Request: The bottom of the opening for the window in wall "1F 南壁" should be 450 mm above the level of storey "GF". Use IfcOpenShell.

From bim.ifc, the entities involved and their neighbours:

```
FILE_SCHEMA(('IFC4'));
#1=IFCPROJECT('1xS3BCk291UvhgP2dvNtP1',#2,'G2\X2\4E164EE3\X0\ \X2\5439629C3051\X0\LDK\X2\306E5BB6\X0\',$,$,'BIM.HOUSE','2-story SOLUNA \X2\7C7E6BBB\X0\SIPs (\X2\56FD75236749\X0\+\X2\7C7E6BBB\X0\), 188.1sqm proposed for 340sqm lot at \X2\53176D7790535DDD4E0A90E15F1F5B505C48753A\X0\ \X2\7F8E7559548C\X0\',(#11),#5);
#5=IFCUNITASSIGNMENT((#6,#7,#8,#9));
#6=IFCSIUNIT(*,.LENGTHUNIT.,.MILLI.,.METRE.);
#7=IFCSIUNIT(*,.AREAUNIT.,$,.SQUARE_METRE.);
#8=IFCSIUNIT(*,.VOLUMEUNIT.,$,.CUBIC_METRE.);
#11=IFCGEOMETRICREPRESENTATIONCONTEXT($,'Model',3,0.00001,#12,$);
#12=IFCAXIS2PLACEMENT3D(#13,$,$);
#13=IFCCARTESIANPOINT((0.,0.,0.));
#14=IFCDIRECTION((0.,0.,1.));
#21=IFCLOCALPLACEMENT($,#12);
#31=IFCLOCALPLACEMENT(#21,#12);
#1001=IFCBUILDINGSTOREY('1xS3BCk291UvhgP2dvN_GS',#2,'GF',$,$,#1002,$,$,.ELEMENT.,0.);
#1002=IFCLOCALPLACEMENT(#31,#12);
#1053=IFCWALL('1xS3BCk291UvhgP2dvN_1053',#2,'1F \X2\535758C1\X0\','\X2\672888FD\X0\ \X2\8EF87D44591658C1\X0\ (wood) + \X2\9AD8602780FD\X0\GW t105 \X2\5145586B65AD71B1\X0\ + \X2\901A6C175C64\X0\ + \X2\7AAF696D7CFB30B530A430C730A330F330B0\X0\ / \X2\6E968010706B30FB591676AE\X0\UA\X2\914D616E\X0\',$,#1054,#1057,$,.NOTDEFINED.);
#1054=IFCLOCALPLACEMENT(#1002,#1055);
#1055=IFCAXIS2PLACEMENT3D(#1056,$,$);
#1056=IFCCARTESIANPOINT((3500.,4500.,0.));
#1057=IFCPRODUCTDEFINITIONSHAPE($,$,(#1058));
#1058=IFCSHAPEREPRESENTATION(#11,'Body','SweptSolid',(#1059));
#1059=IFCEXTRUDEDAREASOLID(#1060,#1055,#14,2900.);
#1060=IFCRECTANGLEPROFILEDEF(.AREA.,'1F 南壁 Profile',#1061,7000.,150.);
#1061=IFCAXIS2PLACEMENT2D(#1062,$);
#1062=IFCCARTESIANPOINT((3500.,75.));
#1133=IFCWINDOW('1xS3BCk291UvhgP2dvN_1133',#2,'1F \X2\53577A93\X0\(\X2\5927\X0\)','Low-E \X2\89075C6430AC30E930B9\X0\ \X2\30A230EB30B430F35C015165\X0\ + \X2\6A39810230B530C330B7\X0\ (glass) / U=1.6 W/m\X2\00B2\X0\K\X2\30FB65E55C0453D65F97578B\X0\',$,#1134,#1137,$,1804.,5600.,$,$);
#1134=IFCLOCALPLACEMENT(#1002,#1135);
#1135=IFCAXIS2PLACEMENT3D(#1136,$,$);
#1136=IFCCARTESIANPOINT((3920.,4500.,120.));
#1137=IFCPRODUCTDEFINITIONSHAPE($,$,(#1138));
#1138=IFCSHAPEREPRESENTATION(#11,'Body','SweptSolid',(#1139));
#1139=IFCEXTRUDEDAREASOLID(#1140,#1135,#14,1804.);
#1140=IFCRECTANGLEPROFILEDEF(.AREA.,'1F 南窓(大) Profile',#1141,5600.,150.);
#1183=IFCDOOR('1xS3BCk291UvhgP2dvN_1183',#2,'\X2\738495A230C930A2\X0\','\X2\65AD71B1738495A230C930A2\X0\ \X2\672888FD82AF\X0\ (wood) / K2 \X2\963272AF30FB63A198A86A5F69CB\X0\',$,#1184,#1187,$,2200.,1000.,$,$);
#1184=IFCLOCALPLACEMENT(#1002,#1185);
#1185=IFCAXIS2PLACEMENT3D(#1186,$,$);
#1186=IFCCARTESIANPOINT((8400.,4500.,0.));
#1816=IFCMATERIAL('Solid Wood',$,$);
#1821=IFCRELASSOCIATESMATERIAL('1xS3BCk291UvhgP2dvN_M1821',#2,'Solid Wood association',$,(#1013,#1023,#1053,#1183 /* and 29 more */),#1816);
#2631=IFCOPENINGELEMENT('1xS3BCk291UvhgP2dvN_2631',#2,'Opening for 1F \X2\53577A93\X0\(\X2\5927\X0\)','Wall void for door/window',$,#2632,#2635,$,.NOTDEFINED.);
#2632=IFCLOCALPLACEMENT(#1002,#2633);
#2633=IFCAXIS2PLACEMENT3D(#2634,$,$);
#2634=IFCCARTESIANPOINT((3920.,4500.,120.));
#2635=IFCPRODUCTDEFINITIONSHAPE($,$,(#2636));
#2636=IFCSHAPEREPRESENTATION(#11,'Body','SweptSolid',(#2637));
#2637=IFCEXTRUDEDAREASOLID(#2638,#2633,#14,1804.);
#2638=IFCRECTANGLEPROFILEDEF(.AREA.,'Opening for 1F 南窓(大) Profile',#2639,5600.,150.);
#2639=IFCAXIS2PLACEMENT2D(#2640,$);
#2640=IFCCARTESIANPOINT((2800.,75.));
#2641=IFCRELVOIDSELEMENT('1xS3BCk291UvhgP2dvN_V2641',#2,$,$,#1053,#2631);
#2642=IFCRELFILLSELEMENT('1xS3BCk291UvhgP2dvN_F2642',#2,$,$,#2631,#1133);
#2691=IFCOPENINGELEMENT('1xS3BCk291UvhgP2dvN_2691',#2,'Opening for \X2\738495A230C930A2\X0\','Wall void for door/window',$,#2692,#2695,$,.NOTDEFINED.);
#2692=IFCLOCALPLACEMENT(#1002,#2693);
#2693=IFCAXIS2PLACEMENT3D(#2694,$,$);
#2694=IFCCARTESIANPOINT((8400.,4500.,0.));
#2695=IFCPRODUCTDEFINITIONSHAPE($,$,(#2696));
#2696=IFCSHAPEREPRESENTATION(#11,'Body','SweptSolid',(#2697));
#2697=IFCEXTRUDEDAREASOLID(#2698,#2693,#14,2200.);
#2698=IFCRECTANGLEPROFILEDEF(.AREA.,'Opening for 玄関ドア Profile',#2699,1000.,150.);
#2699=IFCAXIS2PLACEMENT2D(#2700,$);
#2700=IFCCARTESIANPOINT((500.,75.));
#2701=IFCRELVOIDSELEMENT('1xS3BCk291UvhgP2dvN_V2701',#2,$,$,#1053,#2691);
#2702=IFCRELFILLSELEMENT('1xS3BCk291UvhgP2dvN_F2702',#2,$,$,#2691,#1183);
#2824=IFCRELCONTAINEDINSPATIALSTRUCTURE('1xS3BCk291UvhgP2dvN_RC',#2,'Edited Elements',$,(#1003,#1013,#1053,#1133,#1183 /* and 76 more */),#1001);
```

```python
import numpy as np
import ifcopenshell
import ifcopenshell.api.geometry
import ifcopenshell.geom
import ifcopenshell.util.element
import ifcopenshell.util.placement
import ifcopenshell.util.shape
import ifcopenshell.util.unit

model = ifcopenshell.open("bim.ifc")
unit_scale = ifcopenshell.util.unit.calculate_unit_scale(model)

window = model.by_guid("1xS3BCk291UvhgP2dvN_1133")
opening = window.FillsVoids[0].RelatingOpeningElement
storey = ifcopenshell.util.element.get_container(window, ifc_class="IfcBuildingStorey")
level = ifcopenshell.util.placement.get_local_placement(storey.ObjectPlacement)[2, 3]

# The opening's origin need not be at the sill, so measure its lowest point.
shape = ifcopenshell.geom.create_shape(ifcopenshell.geom.settings(), opening)
bottom = ifcopenshell.util.shape.get_shape_bottom_elevation(shape, shape.geometry) / unit_scale
dz = level + 0.45 / unit_scale - bottom

shift = np.array([0.0, 0.0, dz])
# The window is not placed relative to its opening, so move both.
for product in (opening, window):
    matrix = ifcopenshell.util.placement.get_local_placement(product.ObjectPlacement)
    matrix[:3, 3] += shift
    ifcopenshell.api.geometry.edit_object_placement(model, product=product, matrix=matrix, is_si=False)

print(f"moved by {dz * unit_scale:+.3f} m")

model.write("bim_updated.ifc")
```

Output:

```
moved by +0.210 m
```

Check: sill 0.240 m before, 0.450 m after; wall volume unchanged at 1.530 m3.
